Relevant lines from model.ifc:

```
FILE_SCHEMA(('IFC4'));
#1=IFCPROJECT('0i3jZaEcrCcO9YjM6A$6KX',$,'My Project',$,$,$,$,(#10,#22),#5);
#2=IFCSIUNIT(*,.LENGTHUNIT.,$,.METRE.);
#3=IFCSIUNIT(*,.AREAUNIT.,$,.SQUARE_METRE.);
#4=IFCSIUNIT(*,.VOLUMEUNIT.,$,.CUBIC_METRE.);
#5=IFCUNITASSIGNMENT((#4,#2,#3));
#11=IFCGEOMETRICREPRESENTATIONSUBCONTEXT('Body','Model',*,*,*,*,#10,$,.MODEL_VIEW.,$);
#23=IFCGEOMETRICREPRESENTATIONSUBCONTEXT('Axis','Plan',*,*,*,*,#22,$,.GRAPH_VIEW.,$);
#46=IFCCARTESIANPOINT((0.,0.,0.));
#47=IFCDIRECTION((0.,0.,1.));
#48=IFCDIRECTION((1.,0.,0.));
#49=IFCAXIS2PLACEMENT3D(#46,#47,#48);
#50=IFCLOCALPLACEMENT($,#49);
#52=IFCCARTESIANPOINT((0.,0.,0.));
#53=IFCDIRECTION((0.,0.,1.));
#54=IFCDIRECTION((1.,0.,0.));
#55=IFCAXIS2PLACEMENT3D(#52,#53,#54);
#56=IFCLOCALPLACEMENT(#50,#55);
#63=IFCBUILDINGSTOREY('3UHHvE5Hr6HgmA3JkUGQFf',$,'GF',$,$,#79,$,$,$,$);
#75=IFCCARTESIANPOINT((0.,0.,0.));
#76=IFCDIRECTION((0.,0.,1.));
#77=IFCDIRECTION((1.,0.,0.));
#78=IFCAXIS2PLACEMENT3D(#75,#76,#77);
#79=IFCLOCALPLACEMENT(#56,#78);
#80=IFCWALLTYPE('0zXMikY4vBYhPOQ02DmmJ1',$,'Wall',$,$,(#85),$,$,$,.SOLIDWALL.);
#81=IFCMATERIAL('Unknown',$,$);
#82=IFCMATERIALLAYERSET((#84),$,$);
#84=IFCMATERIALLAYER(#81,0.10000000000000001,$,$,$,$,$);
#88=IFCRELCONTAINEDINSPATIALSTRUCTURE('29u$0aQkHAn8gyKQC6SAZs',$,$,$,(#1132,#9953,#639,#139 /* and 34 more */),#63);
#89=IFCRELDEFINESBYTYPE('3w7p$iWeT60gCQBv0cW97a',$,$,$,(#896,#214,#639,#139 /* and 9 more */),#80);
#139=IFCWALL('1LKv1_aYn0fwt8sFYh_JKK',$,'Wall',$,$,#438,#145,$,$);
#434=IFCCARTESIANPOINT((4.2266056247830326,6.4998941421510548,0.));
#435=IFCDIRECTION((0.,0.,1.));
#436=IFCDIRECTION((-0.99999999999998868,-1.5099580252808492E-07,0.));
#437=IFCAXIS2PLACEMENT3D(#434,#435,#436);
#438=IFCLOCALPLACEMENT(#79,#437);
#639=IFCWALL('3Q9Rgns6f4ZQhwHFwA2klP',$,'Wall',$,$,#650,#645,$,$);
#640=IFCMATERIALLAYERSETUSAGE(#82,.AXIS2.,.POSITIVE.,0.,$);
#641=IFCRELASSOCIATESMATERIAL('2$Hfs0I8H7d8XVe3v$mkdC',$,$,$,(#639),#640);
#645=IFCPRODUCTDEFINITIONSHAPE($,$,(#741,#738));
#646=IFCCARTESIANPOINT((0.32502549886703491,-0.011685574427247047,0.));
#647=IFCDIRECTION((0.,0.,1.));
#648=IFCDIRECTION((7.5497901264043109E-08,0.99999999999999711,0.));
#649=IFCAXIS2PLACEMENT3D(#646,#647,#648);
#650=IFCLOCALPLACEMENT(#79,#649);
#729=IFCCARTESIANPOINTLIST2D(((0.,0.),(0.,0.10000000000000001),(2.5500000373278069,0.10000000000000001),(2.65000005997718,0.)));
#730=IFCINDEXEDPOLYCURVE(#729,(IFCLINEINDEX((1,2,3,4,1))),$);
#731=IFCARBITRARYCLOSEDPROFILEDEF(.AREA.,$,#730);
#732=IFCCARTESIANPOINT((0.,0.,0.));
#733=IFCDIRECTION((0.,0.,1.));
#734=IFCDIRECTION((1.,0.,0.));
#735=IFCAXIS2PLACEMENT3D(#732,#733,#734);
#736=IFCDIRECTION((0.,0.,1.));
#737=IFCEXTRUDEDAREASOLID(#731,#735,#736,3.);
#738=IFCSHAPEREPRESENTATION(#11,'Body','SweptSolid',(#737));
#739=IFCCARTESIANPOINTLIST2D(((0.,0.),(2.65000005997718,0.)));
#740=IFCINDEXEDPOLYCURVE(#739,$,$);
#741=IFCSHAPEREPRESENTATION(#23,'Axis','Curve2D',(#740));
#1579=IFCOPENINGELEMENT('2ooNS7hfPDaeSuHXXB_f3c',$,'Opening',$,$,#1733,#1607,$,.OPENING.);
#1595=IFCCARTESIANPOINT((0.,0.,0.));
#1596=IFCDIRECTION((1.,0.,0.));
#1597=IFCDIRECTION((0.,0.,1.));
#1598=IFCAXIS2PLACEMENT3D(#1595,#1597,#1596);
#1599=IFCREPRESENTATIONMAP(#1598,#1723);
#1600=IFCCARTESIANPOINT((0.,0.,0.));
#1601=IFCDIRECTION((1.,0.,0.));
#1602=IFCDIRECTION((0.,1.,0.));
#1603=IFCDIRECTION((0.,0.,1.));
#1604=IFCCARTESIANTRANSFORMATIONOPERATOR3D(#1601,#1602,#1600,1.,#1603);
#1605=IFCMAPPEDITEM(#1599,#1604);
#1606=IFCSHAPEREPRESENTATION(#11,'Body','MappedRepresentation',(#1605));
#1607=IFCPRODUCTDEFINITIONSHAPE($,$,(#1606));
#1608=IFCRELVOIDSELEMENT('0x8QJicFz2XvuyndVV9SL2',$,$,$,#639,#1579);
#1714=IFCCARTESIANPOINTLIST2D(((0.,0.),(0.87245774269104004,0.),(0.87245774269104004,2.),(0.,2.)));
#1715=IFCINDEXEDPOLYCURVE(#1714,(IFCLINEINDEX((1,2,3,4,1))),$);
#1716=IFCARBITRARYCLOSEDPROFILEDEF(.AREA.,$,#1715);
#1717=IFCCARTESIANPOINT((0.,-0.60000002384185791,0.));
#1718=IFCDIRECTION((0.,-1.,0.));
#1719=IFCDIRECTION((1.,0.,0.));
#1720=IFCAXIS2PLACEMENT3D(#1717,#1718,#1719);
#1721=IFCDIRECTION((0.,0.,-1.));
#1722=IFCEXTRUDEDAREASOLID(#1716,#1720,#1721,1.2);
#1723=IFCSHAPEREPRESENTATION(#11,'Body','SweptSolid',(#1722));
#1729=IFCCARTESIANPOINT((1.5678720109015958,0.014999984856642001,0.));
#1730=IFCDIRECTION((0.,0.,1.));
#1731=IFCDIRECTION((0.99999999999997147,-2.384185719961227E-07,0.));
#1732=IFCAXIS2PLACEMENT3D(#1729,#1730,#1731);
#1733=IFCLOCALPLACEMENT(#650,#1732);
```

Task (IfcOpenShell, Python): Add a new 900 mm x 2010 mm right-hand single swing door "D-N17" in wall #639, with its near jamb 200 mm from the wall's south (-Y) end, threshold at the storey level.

```python
import numpy as np
import ifcopenshell
import ifcopenshell.api.feature
import ifcopenshell.api.geometry
import ifcopenshell.api.root
import ifcopenshell.api.spatial
import ifcopenshell.geom
import ifcopenshell.util.element
import ifcopenshell.util.placement
import ifcopenshell.util.representation
import ifcopenshell.util.shape
import ifcopenshell.util.unit

model = ifcopenshell.open("model.ifc")
unit_scale = ifcopenshell.util.unit.calculate_unit_scale(model)
settings = ifcopenshell.geom.settings()


def volume(element):
    """Net volume in cubic metres, openings subtracted."""
    shape = ifcopenshell.geom.create_shape(settings, element)
    return ifcopenshell.util.shape.get_volume(shape.geometry)


wall = model.by_guid("3Q9Rgns6f4ZQhwHFwA2klP")
storey = ifcopenshell.util.element.get_container(wall, ifc_class="IfcBuildingStorey")
context = ifcopenshell.util.representation.get_context(model, "Model", "Body", "MODEL_VIEW")
before = volume(wall)

width, height, from_end, sill = 0.9, 2.01, 0.2, 0.0  # metres

# The wall runs along its own X axis, and the end named is its -X end.
wall_shape = ifcopenshell.geom.create_shape(settings, wall)
x, y, z = ifcopenshell.util.shape.get_vertices(wall_shape.geometry).T
start = x.min() + from_end
face, thickness = float(y.min()), float(y.max() - y.min())
wall_matrix = ifcopenshell.util.placement.get_local_placement(wall.ObjectPlacement)
level = ifcopenshell.util.placement.get_local_placement(storey.ObjectPlacement)[2, 3]


def in_wall(x, y):
    """Placement at x, y metres in the wall's axes, at sill height."""
    matrix = wall_matrix.copy()
    matrix[:, 3] = wall_matrix @ np.array([x / unit_scale, y / unit_scale, 0.0, 1.0])
    matrix[2, 3] = level + sill / unit_scale
    return matrix


# Opening: a box that overshoots both wall faces by 50 mm.
opening = ifcopenshell.api.root.create_entity(model, ifc_class="IfcOpeningElement", predefined_type="OPENING")
box = ifcopenshell.api.geometry.add_wall_representation(
    model, context=context, length=width, height=height, thickness=thickness + 0.1
)
ifcopenshell.api.geometry.assign_representation(model, product=opening, representation=box)
ifcopenshell.api.geometry.edit_object_placement(model, product=opening, matrix=in_wall(start, face - 0.05), is_si=False)
ifcopenshell.api.feature.add_feature(model, feature=opening, element=wall)

door = ifcopenshell.api.root.create_entity(model, ifc_class="IfcDoor", name="D-N17", predefined_type="DOOR")
door.OverallWidth, door.OverallHeight = width / unit_scale, height / unit_scale
door.OperationType = "SINGLE_SWING_RIGHT"
body = ifcopenshell.api.geometry.add_door_representation(
    model,
    context=context,
    overall_width=door.OverallWidth,
    overall_height=door.OverallHeight,
    operation_type="SINGLE_SWING_RIGHT",
    lining_properties={"LiningDepth": thickness / unit_scale, "ThresholdDepth": thickness / unit_scale},
)
ifcopenshell.api.geometry.assign_representation(model, product=door, representation=body)
ifcopenshell.api.spatial.assign_container(model, products=[door], relating_structure=storey)
ifcopenshell.api.feature.add_filling(model, opening=opening, element=door)

# The lining spans the wall, so the door starts at the wall face.
ifcopenshell.api.geometry.edit_object_placement(model, product=door, matrix=in_wall(start, face), is_si=False)

after = volume(wall)

print(f"wall volume {before:.3f} -> {after:.3f} m3")

model.write("model_updated.ifc")
```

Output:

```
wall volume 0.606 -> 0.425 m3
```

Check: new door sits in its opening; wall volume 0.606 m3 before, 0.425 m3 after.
